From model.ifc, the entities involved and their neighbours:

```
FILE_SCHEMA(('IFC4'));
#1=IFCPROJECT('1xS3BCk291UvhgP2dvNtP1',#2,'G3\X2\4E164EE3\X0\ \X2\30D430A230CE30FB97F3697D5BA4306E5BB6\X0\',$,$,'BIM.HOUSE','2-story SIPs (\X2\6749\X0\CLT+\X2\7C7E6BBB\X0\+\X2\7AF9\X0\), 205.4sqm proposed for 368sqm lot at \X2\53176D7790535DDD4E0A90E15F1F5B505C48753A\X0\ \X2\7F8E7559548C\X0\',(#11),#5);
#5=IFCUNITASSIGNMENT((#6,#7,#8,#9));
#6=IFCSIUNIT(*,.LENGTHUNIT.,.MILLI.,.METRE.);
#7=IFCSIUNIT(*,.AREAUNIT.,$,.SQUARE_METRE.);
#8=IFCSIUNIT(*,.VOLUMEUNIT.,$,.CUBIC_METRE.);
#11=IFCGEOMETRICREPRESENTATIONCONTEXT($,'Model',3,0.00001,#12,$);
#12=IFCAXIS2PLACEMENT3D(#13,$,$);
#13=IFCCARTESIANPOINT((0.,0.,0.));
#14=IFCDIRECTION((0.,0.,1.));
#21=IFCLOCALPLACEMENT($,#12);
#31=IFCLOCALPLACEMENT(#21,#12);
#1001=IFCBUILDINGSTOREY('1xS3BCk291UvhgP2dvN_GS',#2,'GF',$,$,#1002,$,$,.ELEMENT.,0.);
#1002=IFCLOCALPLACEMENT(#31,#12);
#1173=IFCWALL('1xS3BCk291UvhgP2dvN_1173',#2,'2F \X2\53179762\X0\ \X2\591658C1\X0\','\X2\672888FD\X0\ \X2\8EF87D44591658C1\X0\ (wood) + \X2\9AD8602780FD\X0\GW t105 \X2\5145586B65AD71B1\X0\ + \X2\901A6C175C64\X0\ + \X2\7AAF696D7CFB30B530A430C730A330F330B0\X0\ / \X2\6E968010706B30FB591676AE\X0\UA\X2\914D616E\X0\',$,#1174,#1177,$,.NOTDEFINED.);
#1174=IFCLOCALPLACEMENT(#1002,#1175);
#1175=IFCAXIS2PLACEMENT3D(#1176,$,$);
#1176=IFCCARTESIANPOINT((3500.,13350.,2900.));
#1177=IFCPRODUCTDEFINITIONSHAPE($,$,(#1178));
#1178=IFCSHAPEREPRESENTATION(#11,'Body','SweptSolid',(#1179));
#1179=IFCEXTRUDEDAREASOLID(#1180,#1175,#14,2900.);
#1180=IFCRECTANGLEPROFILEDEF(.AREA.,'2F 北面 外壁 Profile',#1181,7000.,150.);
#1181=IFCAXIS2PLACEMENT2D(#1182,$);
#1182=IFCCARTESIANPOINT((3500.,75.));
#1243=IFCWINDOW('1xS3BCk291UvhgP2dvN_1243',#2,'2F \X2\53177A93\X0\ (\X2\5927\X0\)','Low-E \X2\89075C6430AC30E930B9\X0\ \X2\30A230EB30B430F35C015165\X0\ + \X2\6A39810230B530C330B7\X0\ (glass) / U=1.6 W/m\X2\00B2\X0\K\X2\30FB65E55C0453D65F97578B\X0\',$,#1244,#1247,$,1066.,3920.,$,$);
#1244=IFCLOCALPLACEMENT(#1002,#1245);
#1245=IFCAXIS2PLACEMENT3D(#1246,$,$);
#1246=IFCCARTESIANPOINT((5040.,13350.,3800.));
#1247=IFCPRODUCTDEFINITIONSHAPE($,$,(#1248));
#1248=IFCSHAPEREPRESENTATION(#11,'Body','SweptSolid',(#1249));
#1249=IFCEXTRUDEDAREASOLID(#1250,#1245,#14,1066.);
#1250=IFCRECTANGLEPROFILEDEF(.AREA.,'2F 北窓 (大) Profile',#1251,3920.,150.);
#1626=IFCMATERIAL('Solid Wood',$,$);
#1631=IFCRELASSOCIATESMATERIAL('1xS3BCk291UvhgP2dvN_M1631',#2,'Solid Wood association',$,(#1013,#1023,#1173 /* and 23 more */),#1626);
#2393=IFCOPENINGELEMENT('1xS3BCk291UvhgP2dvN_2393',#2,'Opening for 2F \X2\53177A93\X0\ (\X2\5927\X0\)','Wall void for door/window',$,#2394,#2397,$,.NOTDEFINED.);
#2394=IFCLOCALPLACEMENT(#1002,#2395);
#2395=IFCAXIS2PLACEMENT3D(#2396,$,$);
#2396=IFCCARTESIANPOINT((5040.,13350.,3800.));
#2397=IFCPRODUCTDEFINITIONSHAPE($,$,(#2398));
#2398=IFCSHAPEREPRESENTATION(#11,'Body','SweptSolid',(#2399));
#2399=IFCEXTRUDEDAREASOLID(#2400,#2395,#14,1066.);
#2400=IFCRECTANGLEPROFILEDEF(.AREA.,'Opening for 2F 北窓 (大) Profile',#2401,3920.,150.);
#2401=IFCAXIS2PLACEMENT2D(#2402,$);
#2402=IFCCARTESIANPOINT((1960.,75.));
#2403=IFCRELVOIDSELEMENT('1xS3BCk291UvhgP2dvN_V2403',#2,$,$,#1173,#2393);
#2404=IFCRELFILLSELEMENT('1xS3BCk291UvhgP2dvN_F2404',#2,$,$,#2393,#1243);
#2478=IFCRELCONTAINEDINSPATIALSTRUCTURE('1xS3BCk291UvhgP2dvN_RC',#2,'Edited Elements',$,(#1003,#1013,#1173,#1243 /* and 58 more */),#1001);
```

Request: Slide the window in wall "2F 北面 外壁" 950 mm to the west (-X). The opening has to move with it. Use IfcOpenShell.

```python
import ifcopenshell
import ifcopenshell.api.geometry
import ifcopenshell.util.placement
import ifcopenshell.util.unit

model = ifcopenshell.open("model.ifc")
unit_scale = ifcopenshell.util.unit.calculate_unit_scale(model)

window = model.by_guid("1xS3BCk291UvhgP2dvN_1243")
opening = window.FillsVoids[0].RelatingOpeningElement
wall = opening.VoidsElements[0].RelatingBuildingElement

wall_matrix = ifcopenshell.util.placement.get_local_placement(wall.ObjectPlacement)
shift = wall_matrix[:3, 0] * -0.95 / unit_scale
before = ifcopenshell.util.placement.get_local_placement(window.ObjectPlacement)[:3, 3].copy()

# The window is not placed relative to its opening, so move both.
for product in (opening, window):
    matrix = ifcopenshell.util.placement.get_local_placement(product.ObjectPlacement)
    matrix[:3, 3] += shift
    ifcopenshell.api.geometry.edit_object_placement(model, product=product, matrix=matrix, is_si=False)

after = ifcopenshell.util.placement.get_local_placement(window.ObjectPlacement)[:3, 3]
print("window moved by", (after - before).round(3) + 0.0)

model.write("model_updated.ifc")
```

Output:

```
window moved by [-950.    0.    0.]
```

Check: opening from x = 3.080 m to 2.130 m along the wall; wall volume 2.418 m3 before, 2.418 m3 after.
